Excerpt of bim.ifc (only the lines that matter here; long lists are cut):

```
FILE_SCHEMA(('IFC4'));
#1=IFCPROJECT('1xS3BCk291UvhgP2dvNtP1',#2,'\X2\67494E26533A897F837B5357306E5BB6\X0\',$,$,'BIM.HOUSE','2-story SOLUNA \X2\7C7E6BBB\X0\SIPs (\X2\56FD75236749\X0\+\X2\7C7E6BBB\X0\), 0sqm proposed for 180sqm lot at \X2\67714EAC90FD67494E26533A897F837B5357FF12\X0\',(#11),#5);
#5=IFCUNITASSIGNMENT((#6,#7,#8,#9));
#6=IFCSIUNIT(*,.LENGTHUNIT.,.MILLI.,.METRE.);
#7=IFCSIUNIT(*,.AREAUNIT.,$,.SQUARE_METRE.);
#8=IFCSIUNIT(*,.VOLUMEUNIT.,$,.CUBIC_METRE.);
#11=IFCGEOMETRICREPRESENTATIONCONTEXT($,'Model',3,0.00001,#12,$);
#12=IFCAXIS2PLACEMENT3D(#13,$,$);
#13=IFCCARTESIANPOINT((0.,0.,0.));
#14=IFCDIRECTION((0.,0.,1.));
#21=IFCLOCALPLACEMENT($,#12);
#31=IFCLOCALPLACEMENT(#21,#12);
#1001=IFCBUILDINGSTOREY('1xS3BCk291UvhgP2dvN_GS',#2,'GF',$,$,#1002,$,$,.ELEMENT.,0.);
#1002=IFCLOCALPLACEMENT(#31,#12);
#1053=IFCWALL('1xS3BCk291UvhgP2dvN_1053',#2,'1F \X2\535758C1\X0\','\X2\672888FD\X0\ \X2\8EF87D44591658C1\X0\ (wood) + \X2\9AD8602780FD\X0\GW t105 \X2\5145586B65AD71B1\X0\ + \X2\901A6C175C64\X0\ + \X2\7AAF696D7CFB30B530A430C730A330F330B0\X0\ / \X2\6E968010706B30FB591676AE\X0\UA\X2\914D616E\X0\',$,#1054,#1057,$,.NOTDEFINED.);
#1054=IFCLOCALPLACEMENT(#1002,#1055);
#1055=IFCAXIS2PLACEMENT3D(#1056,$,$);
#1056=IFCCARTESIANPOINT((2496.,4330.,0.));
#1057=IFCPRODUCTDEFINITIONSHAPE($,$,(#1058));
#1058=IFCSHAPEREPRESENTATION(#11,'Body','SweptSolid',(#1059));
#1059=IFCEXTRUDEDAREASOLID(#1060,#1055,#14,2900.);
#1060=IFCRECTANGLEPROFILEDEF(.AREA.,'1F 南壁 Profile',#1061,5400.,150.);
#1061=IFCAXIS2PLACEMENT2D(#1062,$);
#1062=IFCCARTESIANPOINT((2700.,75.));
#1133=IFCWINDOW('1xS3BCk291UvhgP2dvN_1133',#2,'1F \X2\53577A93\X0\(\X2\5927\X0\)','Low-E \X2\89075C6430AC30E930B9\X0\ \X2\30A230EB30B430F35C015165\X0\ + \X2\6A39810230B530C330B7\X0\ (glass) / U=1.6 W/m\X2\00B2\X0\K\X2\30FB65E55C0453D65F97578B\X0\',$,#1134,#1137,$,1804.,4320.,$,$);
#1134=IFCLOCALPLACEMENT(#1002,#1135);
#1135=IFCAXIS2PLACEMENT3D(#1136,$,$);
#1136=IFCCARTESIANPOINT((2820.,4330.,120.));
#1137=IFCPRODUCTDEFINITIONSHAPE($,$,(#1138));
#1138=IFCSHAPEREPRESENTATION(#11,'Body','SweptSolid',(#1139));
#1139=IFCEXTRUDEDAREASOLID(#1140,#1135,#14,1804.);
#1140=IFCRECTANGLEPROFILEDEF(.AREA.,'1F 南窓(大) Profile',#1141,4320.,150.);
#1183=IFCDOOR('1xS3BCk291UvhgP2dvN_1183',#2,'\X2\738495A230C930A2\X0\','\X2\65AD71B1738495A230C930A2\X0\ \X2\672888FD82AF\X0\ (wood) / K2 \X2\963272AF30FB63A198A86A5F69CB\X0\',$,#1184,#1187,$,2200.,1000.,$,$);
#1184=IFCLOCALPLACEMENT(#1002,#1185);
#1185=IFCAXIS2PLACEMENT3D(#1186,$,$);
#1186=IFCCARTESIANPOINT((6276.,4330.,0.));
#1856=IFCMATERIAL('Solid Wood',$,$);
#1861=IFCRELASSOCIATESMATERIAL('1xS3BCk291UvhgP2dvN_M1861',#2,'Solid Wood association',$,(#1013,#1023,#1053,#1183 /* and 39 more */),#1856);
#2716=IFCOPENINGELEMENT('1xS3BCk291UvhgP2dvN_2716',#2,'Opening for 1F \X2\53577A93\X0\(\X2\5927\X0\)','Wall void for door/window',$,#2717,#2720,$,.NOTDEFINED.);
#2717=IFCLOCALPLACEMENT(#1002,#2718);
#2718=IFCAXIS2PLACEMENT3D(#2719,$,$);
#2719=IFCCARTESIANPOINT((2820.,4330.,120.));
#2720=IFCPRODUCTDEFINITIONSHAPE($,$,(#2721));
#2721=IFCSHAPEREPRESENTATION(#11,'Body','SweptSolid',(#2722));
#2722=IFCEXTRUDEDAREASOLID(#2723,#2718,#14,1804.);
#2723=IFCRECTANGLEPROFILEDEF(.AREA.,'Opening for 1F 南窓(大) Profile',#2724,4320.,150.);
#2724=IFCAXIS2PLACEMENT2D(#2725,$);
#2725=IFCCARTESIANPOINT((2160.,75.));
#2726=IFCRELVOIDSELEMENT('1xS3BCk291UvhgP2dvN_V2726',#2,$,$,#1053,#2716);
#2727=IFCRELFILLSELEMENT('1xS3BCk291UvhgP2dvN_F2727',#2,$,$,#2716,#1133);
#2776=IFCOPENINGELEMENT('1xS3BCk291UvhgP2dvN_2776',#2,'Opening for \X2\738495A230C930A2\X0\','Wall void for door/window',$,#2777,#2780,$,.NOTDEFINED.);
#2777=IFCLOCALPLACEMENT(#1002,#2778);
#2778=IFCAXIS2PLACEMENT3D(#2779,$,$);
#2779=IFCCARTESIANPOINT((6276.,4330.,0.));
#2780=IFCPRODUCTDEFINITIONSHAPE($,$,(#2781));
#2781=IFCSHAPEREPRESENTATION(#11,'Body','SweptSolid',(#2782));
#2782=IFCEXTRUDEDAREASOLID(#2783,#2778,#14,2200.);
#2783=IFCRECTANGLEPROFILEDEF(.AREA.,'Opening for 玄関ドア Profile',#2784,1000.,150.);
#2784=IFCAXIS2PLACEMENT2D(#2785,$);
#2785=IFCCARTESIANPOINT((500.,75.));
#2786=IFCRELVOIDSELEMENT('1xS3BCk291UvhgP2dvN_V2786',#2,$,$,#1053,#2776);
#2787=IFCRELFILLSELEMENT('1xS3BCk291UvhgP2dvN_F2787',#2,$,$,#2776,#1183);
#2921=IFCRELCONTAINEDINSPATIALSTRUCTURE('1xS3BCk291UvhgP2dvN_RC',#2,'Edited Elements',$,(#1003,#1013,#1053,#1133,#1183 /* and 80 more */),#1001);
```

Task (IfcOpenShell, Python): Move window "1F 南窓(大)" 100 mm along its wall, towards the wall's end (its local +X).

```python
import ifcopenshell
import ifcopenshell.api.geometry
import ifcopenshell.util.placement

model = ifcopenshell.open("bim.ifc")

window = model.by_guid("1xS3BCk291UvhgP2dvN_1133")
opening = window.FillsVoids[0].RelatingOpeningElement
wall = opening.VoidsElements[0].RelatingBuildingElement

wall_matrix = ifcopenshell.util.placement.get_local_placement(wall.ObjectPlacement)
shift = wall_matrix[:3, 0] * 100.0
before = ifcopenshell.util.placement.get_local_placement(window.ObjectPlacement)[:3, 3].copy()

# The window is not placed relative to its opening, so move both.
for product in (opening, window):
    matrix = ifcopenshell.util.placement.get_local_placement(product.ObjectPlacement)
    matrix[:3, 3] += shift
    ifcopenshell.api.geometry.edit_object_placement(model, product=product, matrix=matrix, is_si=False)

after = ifcopenshell.util.placement.get_local_placement(window.ObjectPlacement)[:3, 3]
print("window moved by", (after - before).round(3) + 0.0)

model.write("bim_edited.ifc")
```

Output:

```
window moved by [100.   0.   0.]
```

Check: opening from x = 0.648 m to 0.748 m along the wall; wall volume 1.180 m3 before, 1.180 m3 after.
